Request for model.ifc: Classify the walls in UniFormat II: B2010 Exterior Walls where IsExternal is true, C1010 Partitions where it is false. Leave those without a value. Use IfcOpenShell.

First a look at what the model holds.

```python
import ifcopenshell
import ifcopenshell.util.element

model = ifcopenshell.open("model.ifc")
print(model.schema)
print("classifications:", [c.Name for c in model.by_type("IfcClassification")])
values = [ifcopenshell.util.element.get_pset(e, "Pset_WallCommon", "IsExternal") for e in model.by_type("IfcWall")]
for value in (True, False, None):
    print("IsExternal", value, values.count(value))
```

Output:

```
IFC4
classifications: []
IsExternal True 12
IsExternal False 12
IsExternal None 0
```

```python
import ifcopenshell
import ifcopenshell.api.classification
import ifcopenshell.util.element

model = ifcopenshell.open("model.ifc")

system = ifcopenshell.api.classification.add_classification(model, classification="UniFormat II")

walls = model.by_type("IfcWall")
external = {e: ifcopenshell.util.element.get_pset(e, "Pset_WallCommon", "IsExternal") for e in walls}
for flag, code, name in ((True, "B2010", "Exterior Walls"), (False, "C1010", "Partitions")):
    products = [e for e in walls if external[e] is flag]
    ifcopenshell.api.classification.add_reference(
        model, products=products, classification=system, identification=code, name=name
    )
    print(code, len(products))

model.write("model_updated.ifc")
```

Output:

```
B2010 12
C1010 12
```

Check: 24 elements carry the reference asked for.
